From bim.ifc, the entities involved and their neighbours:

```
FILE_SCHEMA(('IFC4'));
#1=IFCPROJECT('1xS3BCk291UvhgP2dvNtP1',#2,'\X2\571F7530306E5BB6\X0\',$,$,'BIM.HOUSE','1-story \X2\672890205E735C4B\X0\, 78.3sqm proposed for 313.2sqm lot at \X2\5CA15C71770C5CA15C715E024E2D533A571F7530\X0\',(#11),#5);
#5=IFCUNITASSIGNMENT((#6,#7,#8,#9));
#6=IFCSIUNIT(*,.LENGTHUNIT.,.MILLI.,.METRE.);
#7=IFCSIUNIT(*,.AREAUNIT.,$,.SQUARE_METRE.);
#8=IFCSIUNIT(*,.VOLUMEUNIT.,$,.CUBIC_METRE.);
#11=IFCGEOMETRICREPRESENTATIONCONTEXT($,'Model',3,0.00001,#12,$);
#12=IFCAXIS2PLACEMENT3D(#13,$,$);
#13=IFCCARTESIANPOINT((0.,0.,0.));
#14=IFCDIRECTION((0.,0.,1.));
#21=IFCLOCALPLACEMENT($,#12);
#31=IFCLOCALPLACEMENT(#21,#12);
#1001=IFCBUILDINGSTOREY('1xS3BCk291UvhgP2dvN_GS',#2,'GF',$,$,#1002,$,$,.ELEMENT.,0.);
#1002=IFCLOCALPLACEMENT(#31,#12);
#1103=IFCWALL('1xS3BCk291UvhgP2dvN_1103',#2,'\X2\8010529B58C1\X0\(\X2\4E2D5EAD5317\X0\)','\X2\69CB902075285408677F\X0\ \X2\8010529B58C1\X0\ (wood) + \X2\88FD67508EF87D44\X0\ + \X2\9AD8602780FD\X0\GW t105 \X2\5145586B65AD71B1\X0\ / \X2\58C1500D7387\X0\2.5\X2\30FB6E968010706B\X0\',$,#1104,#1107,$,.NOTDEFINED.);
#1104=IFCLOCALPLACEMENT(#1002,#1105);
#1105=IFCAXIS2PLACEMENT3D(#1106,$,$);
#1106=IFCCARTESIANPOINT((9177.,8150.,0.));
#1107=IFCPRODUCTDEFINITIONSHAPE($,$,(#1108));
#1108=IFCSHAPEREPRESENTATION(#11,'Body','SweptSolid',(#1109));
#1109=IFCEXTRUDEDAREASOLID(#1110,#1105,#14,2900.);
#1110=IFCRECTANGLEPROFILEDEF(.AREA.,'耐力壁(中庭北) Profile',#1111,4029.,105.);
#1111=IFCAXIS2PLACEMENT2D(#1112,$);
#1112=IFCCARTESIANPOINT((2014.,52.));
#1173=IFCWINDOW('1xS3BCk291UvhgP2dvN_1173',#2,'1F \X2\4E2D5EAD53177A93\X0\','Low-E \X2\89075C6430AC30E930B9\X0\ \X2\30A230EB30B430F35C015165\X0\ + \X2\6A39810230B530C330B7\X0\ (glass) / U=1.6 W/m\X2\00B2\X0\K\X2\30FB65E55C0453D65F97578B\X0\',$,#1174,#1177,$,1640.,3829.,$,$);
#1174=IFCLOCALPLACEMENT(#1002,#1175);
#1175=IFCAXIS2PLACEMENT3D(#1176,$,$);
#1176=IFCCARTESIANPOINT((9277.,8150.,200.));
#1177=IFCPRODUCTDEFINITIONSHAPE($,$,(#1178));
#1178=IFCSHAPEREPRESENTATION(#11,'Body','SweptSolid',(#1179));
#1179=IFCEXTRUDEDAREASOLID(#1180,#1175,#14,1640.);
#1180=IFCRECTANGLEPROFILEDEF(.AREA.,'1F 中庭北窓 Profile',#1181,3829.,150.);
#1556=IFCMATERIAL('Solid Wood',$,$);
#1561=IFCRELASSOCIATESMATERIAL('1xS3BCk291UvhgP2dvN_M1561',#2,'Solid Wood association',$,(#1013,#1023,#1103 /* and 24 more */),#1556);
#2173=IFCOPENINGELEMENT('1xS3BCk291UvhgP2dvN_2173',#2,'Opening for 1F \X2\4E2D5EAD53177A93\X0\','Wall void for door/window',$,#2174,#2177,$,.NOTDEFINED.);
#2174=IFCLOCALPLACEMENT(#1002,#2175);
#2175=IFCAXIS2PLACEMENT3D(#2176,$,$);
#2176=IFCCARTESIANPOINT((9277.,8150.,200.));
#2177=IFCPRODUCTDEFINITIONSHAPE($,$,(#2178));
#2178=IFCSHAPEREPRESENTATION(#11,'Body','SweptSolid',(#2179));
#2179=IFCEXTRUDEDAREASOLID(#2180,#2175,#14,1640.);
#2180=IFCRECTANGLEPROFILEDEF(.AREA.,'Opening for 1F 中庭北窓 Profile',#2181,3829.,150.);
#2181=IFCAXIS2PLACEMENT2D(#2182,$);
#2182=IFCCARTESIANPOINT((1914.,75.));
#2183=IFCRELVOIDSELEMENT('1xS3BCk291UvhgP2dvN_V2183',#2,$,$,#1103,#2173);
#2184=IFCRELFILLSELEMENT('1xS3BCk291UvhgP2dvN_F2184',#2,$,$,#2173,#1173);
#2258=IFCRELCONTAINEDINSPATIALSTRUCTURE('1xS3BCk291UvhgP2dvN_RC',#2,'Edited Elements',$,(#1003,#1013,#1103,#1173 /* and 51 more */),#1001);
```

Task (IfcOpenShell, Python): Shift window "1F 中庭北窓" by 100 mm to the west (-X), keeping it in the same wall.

```python
import ifcopenshell
import ifcopenshell.api.geometry
import ifcopenshell.util.placement
import ifcopenshell.util.unit

model = ifcopenshell.open("bim.ifc")
unit_scale = ifcopenshell.util.unit.calculate_unit_scale(model)

window = model.by_guid("1xS3BCk291UvhgP2dvN_1173")
opening = window.FillsVoids[0].RelatingOpeningElement
wall = opening.VoidsElements[0].RelatingBuildingElement

wall_matrix = ifcopenshell.util.placement.get_local_placement(wall.ObjectPlacement)
shift = wall_matrix[:3, 0] * -0.1 / unit_scale
before = ifcopenshell.util.placement.get_local_placement(window.ObjectPlacement)[:3, 3].copy()

# The window is not placed relative to its opening, so move both.
for product in (opening, window):
    matrix = ifcopenshell.util.placement.get_local_placement(product.ObjectPlacement)
    matrix[:3, 3] += shift
    ifcopenshell.api.geometry.edit_object_placement(model, product=product, matrix=matrix, is_si=False)

after = ifcopenshell.util.placement.get_local_placement(window.ObjectPlacement)[:3, 3]
print("window moved by", (after - before).round(3) + 0.0)

model.write("bim_updated.ifc")
```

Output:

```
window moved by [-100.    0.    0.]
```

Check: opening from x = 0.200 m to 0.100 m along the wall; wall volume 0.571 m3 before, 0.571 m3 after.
